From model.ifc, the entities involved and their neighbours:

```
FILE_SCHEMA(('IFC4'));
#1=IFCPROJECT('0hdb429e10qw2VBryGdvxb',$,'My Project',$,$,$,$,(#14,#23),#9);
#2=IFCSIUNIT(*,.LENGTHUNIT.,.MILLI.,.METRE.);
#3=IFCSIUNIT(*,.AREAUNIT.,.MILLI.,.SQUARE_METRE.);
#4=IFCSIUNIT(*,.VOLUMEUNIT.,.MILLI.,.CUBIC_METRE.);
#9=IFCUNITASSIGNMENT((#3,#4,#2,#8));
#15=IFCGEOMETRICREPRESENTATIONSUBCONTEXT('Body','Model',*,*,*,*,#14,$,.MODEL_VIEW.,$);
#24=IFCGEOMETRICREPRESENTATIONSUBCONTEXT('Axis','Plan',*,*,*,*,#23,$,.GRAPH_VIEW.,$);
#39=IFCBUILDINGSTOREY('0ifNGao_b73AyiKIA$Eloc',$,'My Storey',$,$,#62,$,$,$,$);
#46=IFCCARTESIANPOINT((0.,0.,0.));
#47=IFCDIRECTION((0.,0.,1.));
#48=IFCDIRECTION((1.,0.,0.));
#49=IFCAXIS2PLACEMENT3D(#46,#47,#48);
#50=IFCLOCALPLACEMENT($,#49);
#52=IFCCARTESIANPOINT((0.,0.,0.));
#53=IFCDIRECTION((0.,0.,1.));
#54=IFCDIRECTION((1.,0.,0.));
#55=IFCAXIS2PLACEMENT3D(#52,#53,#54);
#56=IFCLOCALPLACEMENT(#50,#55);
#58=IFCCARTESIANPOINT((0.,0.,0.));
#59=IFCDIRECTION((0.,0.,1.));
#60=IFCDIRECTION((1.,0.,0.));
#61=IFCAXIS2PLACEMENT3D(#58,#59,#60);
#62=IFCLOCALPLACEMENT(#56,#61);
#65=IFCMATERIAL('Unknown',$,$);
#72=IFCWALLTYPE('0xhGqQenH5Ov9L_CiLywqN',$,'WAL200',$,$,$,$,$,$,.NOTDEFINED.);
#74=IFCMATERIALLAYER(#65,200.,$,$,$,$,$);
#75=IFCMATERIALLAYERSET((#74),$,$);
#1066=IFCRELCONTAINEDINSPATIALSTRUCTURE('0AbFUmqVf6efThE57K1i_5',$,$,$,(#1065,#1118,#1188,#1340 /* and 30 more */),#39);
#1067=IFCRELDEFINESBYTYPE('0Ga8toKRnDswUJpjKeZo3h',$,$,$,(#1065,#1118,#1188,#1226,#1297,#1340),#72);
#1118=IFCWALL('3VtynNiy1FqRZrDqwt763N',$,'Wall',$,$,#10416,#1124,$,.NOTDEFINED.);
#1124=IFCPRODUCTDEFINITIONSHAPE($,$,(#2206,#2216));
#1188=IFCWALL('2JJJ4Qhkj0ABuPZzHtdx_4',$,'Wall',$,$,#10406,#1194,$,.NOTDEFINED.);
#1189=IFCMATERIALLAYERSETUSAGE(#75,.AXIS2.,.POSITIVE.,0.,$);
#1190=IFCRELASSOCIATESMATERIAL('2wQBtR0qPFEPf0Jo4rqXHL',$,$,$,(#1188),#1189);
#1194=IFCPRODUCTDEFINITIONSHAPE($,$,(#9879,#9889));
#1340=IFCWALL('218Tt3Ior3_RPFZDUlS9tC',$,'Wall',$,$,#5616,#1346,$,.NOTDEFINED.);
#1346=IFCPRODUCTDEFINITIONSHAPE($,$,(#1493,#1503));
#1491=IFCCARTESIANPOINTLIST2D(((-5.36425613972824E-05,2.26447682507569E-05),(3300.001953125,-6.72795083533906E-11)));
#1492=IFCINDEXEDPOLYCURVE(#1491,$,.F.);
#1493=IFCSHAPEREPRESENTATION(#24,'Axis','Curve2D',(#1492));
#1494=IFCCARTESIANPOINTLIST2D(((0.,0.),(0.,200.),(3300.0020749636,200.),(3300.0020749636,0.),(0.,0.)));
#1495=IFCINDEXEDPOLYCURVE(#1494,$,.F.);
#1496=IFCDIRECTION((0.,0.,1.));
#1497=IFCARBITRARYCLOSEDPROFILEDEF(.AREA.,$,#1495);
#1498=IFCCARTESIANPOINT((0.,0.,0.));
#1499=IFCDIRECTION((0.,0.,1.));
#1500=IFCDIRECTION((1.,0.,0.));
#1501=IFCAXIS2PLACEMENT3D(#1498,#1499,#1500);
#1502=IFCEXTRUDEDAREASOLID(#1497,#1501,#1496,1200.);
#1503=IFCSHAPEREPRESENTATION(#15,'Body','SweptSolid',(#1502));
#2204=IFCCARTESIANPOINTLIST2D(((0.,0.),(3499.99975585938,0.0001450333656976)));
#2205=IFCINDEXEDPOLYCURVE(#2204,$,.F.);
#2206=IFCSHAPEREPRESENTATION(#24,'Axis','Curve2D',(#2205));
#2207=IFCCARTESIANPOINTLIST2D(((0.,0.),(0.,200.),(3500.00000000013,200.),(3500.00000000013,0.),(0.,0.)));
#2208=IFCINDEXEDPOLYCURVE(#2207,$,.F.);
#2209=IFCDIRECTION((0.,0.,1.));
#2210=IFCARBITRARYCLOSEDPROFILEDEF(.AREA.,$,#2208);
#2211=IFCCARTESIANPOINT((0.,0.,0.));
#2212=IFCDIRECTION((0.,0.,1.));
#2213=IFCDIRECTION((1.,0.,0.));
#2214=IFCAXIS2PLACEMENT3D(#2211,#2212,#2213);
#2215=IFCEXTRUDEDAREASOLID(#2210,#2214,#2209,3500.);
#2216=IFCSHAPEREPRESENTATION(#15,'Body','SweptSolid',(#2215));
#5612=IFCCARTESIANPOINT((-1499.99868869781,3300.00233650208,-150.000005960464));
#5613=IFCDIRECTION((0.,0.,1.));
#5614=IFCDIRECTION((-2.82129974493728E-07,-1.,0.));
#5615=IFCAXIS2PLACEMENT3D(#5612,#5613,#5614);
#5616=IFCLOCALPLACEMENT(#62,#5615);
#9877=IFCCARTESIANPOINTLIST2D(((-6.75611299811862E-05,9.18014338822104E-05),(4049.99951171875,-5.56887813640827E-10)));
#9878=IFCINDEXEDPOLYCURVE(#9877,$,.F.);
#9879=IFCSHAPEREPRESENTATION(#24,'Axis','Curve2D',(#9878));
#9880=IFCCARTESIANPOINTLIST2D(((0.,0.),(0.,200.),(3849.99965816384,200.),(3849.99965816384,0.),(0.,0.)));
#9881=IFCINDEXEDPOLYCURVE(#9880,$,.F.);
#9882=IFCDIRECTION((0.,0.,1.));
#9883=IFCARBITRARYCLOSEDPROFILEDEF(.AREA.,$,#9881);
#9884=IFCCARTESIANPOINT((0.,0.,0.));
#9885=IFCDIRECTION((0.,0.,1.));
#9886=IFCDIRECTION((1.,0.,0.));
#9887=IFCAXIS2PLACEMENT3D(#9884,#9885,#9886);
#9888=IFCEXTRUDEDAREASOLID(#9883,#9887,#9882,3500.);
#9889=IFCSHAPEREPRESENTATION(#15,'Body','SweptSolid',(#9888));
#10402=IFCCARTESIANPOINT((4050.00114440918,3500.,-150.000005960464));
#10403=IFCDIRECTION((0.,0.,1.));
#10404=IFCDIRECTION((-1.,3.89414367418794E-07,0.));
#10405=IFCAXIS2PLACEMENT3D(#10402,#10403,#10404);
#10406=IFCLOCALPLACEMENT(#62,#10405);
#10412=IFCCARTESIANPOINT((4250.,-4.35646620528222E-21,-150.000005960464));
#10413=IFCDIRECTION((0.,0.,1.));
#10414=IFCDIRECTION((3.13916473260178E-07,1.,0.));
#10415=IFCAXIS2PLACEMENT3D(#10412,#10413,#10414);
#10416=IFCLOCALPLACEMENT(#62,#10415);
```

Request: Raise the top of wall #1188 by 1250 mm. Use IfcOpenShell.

```python
import ifcopenshell
import ifcopenshell.geom
import ifcopenshell.util.representation
import ifcopenshell.util.shape

model = ifcopenshell.open("model.ifc")
settings = ifcopenshell.geom.settings()


def volume(element):
    """Net volume in cubic metres, openings subtracted."""
    shape = ifcopenshell.geom.create_shape(settings, element)
    return ifcopenshell.util.shape.get_volume(shape.geometry)


wall = model.by_guid("2JJJ4Qhkj0ABuPZzHtdx_4")
before = volume(wall)

body = ifcopenshell.util.representation.get_representation(wall, "Model", "Body")
solid = body.Items[0]
old_height = solid.Depth
solid.Depth += 1250.0
after = volume(wall)

print(f"height {old_height:g} -> {solid.Depth:g}, volume {before:.3f} -> {after:.3f} m3")

model.write("model_rev.ifc")
```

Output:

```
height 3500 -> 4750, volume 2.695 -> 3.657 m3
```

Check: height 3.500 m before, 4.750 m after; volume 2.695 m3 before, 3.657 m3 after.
